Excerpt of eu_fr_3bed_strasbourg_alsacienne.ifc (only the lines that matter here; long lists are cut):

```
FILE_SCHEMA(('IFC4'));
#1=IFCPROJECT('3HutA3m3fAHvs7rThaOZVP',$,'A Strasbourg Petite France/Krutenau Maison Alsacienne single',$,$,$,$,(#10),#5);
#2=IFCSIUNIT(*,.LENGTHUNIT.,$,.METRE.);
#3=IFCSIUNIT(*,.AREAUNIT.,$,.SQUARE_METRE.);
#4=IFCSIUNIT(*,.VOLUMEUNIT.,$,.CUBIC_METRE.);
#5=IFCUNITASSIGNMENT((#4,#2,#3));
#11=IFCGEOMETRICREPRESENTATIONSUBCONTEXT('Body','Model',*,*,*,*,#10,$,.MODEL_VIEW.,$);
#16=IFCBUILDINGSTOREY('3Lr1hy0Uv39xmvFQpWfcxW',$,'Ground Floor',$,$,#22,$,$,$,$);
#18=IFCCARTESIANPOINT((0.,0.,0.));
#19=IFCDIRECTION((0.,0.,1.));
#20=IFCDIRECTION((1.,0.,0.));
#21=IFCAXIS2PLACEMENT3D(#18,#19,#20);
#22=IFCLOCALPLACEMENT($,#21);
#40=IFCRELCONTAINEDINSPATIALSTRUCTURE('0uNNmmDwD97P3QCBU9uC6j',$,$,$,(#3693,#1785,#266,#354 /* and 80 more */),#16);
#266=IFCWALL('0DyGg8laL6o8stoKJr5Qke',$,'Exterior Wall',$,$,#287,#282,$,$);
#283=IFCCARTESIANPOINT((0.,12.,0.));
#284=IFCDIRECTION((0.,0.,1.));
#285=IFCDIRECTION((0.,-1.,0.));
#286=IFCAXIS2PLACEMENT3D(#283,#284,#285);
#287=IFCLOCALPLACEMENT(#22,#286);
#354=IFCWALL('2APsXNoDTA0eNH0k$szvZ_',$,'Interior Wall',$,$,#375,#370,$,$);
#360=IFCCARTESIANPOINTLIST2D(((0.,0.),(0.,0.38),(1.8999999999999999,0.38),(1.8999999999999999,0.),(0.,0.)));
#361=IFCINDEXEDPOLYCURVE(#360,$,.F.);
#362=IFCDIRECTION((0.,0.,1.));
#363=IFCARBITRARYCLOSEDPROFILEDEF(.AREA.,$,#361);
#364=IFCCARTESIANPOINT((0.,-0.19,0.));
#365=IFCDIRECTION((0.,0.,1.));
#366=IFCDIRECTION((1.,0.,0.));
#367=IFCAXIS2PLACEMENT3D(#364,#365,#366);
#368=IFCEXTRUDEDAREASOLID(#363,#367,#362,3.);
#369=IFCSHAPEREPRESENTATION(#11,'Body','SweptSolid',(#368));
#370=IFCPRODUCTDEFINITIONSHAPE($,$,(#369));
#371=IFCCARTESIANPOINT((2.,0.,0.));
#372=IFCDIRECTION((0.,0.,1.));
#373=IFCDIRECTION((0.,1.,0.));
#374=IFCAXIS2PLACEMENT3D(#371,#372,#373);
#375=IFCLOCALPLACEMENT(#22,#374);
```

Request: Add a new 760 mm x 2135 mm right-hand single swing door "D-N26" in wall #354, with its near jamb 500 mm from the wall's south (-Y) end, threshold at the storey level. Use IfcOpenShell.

```python
import numpy as np
import ifcopenshell
import ifcopenshell.api.feature
import ifcopenshell.api.geometry
import ifcopenshell.api.root
import ifcopenshell.api.spatial
import ifcopenshell.geom
import ifcopenshell.util.element
import ifcopenshell.util.placement
import ifcopenshell.util.representation
import ifcopenshell.util.shape
import ifcopenshell.util.unit

model = ifcopenshell.open("eu_fr_3bed_strasbourg_alsacienne.ifc")
unit_scale = ifcopenshell.util.unit.calculate_unit_scale(model)
settings = ifcopenshell.geom.settings()


def volume(element):
    """Net volume in cubic metres, openings subtracted."""
    shape = ifcopenshell.geom.create_shape(settings, element)
    return ifcopenshell.util.shape.get_volume(shape.geometry)


wall = model.by_id(354)
storey = ifcopenshell.util.element.get_container(wall, ifc_class="IfcBuildingStorey")
context = ifcopenshell.util.representation.get_context(model, "Model", "Body", "MODEL_VIEW")
before = volume(wall)

width, height, from_end, sill = 0.76, 2.135, 0.5, 0.0  # metres

# The wall runs along its own X axis, and the end named is its -X end.
wall_shape = ifcopenshell.geom.create_shape(settings, wall)
x, y, z = ifcopenshell.util.shape.get_vertices(wall_shape.geometry).T
start = x.min() + from_end
face, thickness = float(y.min()), float(y.max() - y.min())
wall_matrix = ifcopenshell.util.placement.get_local_placement(wall.ObjectPlacement)
level = ifcopenshell.util.placement.get_local_placement(storey.ObjectPlacement)[2, 3]


def in_wall(x, y):
    """Placement at x, y metres in the wall's axes, at sill height."""
    matrix = wall_matrix.copy()
    matrix[:, 3] = wall_matrix @ np.array([x / unit_scale, y / unit_scale, 0.0, 1.0])
    matrix[2, 3] = level + sill / unit_scale
    return matrix


# Opening: a box that overshoots both wall faces by 50 mm.
opening = ifcopenshell.api.root.create_entity(model, ifc_class="IfcOpeningElement", predefined_type="OPENING")
box = ifcopenshell.api.geometry.add_wall_representation(
    model, context=context, length=width, height=height, thickness=thickness + 0.1
)
ifcopenshell.api.geometry.assign_representation(model, product=opening, representation=box)
ifcopenshell.api.geometry.edit_object_placement(model, product=opening, matrix=in_wall(start, face - 0.05), is_si=False)
ifcopenshell.api.feature.add_feature(model, feature=opening, element=wall)

door = ifcopenshell.api.root.create_entity(model, ifc_class="IfcDoor", name="D-N26", predefined_type="DOOR")
door.OverallWidth, door.OverallHeight = width / unit_scale, height / unit_scale
door.OperationType = "SINGLE_SWING_RIGHT"
body = ifcopenshell.api.geometry.add_door_representation(
    model,
    context=context,
    overall_width=door.OverallWidth,
    overall_height=door.OverallHeight,
    operation_type="SINGLE_SWING_RIGHT",
    lining_properties={"LiningDepth": thickness / unit_scale, "ThresholdDepth": thickness / unit_scale},
)
ifcopenshell.api.geometry.assign_representation(model, product=door, representation=body)
ifcopenshell.api.spatial.assign_container(model, products=[door], relating_structure=storey)
ifcopenshell.api.feature.add_filling(model, opening=opening, element=door)

# The lining spans the wall, so the door starts at the wall face.
ifcopenshell.api.geometry.edit_object_placement(model, product=door, matrix=in_wall(start, face), is_si=False)

after = volume(wall)

print(f"wall volume {before:.3f} -> {after:.3f} m3")

model.write("eu_fr_3bed_strasbourg_alsacienne_v2.ifc")
```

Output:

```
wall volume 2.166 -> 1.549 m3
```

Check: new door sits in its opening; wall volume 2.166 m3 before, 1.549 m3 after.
